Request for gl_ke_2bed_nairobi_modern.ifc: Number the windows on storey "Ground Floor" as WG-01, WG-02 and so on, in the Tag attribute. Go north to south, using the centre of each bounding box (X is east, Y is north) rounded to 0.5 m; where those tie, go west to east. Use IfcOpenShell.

First a look at what the model holds.

```python
import ifcopenshell
import ifcopenshell.util.element
import ifcopenshell.util.placement

model = ifcopenshell.open("gl_ke_2bed_nairobi_modern.ifc")
print(model.schema)
storey = next(s for s in model.by_type("IfcBuildingStorey") if s.Name == "Ground Floor")
windows = [e for e in ifcopenshell.util.element.get_decomposition(storey) if e.is_a("IfcWindow")]
for e in sorted(windows, key=lambda e: e.id()):
    origin = ifcopenshell.util.placement.get_local_placement(e.ObjectPlacement)[:3, 3]
    print(e.id(), e.Tag, e.Name, origin.round(2) + 0.0, sep=" | ")
```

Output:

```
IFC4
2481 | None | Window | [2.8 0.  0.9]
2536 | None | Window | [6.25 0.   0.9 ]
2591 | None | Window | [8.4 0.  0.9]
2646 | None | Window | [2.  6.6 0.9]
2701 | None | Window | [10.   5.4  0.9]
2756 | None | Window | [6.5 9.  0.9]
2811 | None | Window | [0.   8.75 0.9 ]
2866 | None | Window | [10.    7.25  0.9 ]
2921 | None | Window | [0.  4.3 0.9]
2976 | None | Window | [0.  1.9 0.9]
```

```python
import ifcopenshell
import ifcopenshell.geom
import ifcopenshell.util.element
import ifcopenshell.util.shape

model = ifcopenshell.open("gl_ke_2bed_nairobi_modern.ifc")
settings = ifcopenshell.geom.settings()
settings.set("use-world-coords", True)


def centre(element):
    shape = ifcopenshell.geom.create_shape(settings, element)
    return ifcopenshell.util.shape.get_bbox_centroid(shape.geometry)


storey = next(s for s in model.by_type("IfcBuildingStorey") if s.Name == "Ground Floor")
windows = [e for e in ifcopenshell.util.element.get_decomposition(storey) if e.is_a("IfcWindow")]

# Insertion points can sit at a corner or the storey origin, so sort by the geometry (in metres).
centres = {e: centre(e) for e in windows}
windows.sort(key=lambda e: (-round(centres[e][1] / 0.5), centres[e][0]))

for i, e in enumerate(windows, start=1):
    number = f"WG-{i:02d}"
    e.Tag = number
    print(e.id(), number)

model.write("gl_ke_2bed_nairobi_modern_updated.ifc")
```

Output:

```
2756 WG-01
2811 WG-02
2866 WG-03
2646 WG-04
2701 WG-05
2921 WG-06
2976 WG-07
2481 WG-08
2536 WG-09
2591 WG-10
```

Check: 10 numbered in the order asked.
